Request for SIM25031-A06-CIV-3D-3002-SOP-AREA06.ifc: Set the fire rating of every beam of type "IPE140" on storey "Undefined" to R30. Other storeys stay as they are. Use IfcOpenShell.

First a look at what the model holds.

```python
import ifcopenshell
import ifcopenshell.util.element

model = ifcopenshell.open("SIM25031-A06-CIV-3D-3002-SOP-AREA06.ifc")
print(model.schema)
storey = next(s for s in model.by_type("IfcBuildingStorey") if s.Name == "Undefined")
beams = [e for e in ifcopenshell.util.element.get_decomposition(storey) if e.is_a("IfcBeam")]
seen = {}
for e in beams:
    element_type = ifcopenshell.util.element.get_type(e)
    key = (element_type.Name if element_type != e and element_type else None, ifcopenshell.util.element.get_pset(e, "Pset_BeamCommon", "FireRating"))
    seen[key] = seen.get(key, 0) + 1
for (name, value), count in sorted(seen.items(), key=str):
    print(count, "x", name, "|", value)
```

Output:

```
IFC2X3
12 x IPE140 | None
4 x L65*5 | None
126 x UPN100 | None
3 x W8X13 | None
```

```python
import ifcopenshell
import ifcopenshell.api.pset
import ifcopenshell.util.element

model = ifcopenshell.open("SIM25031-A06-CIV-3D-3002-SOP-AREA06.ifc")

storey = next(s for s in model.by_type("IfcBuildingStorey") if s.Name == "Undefined")
beams = [e for e in ifcopenshell.util.element.get_decomposition(storey) if e.is_a("IfcBeam")]

count = 0
for e in beams:
    element_type = ifcopenshell.util.element.get_type(e)
    if element_type in (None, e) or element_type.Name != "IPE140":
        continue
    found = ifcopenshell.util.element.get_pset(e, "Pset_BeamCommon", should_inherit=False)
    if found:
        pset = model.by_id(found["id"])
        if len(ifcopenshell.util.element.get_elements_by_pset(pset)) > 1:
            pset = ifcopenshell.api.pset.unshare_pset(model, products=[e], pset=pset)[0]
    else:
        pset = ifcopenshell.api.pset.add_pset(model, product=e, name="Pset_BeamCommon")
    ifcopenshell.api.pset.edit_pset(model, pset=pset, properties={"FireRating": "R30"})
    count += 1

print(count, "beams updated")

model.write("SIM25031-A06-CIV-3D-3002-SOP-AREA06-out.ifc")
```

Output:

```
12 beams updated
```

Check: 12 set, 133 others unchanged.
